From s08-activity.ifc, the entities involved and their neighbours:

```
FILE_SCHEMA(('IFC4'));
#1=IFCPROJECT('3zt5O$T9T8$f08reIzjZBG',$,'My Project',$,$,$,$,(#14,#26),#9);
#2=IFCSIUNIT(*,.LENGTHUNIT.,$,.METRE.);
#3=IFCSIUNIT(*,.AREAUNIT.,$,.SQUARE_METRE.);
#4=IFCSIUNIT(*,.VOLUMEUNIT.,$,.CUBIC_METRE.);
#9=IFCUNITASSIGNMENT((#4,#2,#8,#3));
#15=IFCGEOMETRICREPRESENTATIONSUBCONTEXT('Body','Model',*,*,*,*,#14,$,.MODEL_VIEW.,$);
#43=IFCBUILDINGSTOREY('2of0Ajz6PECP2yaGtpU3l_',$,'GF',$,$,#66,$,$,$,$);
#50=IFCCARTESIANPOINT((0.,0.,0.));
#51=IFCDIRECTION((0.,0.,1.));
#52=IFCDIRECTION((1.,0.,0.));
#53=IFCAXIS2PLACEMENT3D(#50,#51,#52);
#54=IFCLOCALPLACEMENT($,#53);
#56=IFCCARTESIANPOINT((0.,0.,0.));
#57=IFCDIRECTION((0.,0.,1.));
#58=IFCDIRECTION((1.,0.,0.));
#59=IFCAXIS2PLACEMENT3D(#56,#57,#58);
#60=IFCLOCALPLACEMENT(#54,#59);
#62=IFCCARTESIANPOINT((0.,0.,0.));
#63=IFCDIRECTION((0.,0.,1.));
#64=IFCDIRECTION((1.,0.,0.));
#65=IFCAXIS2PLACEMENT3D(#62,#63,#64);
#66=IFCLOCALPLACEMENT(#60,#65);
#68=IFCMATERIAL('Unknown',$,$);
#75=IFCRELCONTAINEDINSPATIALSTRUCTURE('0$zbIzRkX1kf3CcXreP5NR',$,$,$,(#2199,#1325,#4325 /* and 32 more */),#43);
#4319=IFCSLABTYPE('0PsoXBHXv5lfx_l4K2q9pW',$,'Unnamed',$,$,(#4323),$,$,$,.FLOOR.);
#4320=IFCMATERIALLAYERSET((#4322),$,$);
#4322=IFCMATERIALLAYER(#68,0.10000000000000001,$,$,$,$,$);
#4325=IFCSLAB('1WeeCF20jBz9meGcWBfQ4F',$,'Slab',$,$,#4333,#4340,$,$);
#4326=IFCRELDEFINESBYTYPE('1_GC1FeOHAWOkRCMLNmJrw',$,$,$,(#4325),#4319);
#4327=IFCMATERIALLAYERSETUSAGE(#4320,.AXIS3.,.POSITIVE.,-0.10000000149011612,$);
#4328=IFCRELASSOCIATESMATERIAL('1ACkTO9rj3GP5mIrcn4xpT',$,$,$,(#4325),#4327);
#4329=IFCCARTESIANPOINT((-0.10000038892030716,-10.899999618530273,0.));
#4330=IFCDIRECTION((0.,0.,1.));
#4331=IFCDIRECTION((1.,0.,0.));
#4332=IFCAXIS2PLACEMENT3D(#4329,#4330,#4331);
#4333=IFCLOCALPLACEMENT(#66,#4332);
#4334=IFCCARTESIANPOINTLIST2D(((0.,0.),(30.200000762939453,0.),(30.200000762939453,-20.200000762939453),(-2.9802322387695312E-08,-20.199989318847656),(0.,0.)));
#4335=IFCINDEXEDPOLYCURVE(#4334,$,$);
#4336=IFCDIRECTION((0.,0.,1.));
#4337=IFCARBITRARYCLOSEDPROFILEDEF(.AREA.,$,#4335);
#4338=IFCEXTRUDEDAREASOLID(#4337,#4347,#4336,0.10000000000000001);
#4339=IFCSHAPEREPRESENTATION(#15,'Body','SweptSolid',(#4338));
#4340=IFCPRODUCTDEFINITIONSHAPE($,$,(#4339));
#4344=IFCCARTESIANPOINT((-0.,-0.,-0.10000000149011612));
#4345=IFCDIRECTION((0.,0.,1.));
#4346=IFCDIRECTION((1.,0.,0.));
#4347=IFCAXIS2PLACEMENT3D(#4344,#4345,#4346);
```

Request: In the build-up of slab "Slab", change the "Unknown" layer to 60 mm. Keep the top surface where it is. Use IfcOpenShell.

```python
import ifcopenshell
import ifcopenshell.util.element
import ifcopenshell.util.representation
import ifcopenshell.util.unit

model = ifcopenshell.open("s08-activity.ifc")
unit_scale = ifcopenshell.util.unit.calculate_unit_scale(model)

layer_set = model.by_id(4320)
layer = next(l for l in layer_set.MaterialLayers if l.Material and l.Material.Name == "Unknown")
change = 0.06 / unit_scale - layer.LayerThickness
layer.LayerThickness += change

# Geometry does not follow the layer set by itself.
slabs = [e for e in ifcopenshell.util.element.get_elements_by_material(model, layer_set) if e.is_a("IfcSlab")]
for slab in sorted(slabs, key=lambda e: e.id()):
    body = ifcopenshell.util.representation.get_representation(slab, "Model", "Body")
    solid = body.Items[0]
    old_depth = solid.Depth
    solid.Depth += change
    # Extruded upwards: lower the start of the extrusion so the top stays.
    x, y, z = solid.Position.Location.Coordinates
    solid.Position.Location = model.createIfcCartesianPoint((x, y, z - change))
    print(slab.id(), f"{old_depth:g} -> {solid.Depth:g}")

# The layers are counted up from the underside, which has moved.
for usage in {ifcopenshell.util.element.get_material(slab) for slab in slabs}:
    usage.OffsetFromReferenceLine -= change

model.write("s08-activity_v2.ifc")
```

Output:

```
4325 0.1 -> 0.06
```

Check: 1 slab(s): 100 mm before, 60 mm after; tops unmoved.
